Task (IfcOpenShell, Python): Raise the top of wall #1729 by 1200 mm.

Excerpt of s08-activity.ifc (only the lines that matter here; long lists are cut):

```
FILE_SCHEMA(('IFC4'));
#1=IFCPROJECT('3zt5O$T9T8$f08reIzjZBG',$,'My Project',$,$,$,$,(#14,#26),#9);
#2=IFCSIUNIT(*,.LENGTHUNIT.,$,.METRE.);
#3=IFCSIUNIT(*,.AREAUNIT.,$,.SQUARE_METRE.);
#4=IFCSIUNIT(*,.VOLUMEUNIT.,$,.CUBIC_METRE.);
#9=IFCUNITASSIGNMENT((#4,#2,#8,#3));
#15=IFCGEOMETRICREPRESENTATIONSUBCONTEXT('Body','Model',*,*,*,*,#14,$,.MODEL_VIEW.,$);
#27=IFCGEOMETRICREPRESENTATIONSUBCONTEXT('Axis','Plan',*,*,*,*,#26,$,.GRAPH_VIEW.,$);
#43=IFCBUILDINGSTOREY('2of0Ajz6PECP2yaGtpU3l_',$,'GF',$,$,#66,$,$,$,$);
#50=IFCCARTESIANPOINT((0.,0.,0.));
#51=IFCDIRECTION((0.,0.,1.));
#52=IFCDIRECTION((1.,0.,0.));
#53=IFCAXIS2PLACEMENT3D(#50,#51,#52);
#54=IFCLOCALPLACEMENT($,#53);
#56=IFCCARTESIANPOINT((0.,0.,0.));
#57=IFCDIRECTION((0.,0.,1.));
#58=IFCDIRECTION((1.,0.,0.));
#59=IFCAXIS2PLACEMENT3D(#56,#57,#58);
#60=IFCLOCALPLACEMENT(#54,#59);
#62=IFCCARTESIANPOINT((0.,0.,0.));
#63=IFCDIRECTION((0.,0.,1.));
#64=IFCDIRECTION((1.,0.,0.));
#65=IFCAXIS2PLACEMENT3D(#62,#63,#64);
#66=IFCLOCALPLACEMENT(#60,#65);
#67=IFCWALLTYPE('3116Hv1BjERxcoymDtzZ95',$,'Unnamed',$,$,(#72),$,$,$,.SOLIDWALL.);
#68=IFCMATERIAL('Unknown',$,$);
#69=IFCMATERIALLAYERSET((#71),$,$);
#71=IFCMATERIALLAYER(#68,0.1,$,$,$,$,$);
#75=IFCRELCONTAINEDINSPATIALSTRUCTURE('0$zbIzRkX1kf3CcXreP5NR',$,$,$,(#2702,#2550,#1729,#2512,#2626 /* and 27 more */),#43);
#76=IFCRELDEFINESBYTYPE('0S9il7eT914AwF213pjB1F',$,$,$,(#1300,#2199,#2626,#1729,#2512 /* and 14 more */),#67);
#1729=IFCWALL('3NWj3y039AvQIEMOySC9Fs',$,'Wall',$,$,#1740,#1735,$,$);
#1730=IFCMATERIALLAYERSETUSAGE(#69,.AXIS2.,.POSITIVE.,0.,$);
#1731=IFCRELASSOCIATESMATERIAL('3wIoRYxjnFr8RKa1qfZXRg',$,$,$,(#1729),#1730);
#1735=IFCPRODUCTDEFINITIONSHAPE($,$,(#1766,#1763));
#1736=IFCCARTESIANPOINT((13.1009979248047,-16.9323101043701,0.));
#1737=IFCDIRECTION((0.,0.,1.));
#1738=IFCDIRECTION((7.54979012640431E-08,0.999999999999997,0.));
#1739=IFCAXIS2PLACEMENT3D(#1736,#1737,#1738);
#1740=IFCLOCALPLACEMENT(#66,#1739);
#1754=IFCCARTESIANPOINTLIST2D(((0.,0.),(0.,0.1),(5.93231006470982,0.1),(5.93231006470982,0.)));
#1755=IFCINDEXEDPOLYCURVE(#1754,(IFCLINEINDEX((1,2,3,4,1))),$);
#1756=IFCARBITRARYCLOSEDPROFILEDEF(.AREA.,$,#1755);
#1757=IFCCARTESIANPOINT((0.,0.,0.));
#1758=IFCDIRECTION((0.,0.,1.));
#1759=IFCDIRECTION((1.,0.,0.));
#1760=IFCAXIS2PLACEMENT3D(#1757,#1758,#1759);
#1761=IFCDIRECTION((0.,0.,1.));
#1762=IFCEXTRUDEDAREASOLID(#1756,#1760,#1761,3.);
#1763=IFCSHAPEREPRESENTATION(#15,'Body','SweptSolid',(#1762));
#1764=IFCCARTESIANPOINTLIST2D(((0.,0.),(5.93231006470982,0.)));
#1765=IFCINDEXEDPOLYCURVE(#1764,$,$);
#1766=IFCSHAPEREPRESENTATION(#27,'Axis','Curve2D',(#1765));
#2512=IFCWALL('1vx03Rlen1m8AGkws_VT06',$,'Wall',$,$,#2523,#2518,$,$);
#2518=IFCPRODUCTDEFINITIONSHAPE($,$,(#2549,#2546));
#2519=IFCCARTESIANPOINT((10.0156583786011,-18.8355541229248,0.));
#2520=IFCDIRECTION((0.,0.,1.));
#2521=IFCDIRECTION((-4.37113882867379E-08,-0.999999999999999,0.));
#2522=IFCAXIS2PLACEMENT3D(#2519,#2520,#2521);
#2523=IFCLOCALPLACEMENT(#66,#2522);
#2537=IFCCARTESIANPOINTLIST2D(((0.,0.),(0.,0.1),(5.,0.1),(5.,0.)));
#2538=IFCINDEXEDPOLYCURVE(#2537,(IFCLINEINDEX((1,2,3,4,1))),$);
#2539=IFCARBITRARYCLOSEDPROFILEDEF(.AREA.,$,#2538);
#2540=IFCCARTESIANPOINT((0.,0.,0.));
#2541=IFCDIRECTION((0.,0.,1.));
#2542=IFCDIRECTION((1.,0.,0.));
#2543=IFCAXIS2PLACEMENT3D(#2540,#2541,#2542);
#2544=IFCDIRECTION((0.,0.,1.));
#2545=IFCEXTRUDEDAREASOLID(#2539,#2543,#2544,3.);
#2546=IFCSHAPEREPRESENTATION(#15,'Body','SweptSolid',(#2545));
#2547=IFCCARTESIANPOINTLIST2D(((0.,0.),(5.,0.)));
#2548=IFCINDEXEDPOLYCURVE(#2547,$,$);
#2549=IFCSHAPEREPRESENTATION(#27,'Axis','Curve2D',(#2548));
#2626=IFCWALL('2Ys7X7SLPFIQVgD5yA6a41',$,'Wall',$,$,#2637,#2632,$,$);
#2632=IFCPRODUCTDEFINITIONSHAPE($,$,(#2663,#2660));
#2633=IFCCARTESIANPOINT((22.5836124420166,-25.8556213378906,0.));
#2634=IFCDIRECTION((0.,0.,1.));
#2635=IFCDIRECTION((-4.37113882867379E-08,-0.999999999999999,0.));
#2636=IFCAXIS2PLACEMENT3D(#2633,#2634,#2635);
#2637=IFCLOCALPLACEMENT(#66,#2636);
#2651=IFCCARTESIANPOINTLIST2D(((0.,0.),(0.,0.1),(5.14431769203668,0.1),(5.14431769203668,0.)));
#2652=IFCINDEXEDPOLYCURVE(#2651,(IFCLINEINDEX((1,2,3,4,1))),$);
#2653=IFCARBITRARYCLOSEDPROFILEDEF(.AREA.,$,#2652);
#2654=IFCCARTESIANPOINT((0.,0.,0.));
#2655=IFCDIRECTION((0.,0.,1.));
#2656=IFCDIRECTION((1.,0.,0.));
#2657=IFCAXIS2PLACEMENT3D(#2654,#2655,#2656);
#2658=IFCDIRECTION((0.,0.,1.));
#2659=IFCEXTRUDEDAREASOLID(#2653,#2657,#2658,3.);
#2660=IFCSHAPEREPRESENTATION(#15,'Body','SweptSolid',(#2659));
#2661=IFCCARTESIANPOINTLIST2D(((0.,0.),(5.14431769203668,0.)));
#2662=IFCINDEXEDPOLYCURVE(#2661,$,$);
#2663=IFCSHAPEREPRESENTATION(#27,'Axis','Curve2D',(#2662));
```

```python
import ifcopenshell
import ifcopenshell.geom
import ifcopenshell.util.representation
import ifcopenshell.util.shape
import ifcopenshell.util.unit

model = ifcopenshell.open("s08-activity.ifc")
unit_scale = ifcopenshell.util.unit.calculate_unit_scale(model)
settings = ifcopenshell.geom.settings()


def volume(element):
    """Net volume in cubic metres, openings subtracted."""
    shape = ifcopenshell.geom.create_shape(settings, element)
    return ifcopenshell.util.shape.get_volume(shape.geometry)


wall = model.by_guid("3NWj3y039AvQIEMOySC9Fs")
before = volume(wall)

body = ifcopenshell.util.representation.get_representation(wall, "Model", "Body")
solid = body.Items[0]
old_height = solid.Depth
solid.Depth += 1.2 / unit_scale
after = volume(wall)

print(f"height {old_height:g} -> {solid.Depth:g}, volume {before:.3f} -> {after:.3f} m3")

model.write("s08-activity_rev.ifc")
```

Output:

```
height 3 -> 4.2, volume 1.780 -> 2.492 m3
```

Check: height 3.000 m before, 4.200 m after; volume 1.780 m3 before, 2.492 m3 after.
